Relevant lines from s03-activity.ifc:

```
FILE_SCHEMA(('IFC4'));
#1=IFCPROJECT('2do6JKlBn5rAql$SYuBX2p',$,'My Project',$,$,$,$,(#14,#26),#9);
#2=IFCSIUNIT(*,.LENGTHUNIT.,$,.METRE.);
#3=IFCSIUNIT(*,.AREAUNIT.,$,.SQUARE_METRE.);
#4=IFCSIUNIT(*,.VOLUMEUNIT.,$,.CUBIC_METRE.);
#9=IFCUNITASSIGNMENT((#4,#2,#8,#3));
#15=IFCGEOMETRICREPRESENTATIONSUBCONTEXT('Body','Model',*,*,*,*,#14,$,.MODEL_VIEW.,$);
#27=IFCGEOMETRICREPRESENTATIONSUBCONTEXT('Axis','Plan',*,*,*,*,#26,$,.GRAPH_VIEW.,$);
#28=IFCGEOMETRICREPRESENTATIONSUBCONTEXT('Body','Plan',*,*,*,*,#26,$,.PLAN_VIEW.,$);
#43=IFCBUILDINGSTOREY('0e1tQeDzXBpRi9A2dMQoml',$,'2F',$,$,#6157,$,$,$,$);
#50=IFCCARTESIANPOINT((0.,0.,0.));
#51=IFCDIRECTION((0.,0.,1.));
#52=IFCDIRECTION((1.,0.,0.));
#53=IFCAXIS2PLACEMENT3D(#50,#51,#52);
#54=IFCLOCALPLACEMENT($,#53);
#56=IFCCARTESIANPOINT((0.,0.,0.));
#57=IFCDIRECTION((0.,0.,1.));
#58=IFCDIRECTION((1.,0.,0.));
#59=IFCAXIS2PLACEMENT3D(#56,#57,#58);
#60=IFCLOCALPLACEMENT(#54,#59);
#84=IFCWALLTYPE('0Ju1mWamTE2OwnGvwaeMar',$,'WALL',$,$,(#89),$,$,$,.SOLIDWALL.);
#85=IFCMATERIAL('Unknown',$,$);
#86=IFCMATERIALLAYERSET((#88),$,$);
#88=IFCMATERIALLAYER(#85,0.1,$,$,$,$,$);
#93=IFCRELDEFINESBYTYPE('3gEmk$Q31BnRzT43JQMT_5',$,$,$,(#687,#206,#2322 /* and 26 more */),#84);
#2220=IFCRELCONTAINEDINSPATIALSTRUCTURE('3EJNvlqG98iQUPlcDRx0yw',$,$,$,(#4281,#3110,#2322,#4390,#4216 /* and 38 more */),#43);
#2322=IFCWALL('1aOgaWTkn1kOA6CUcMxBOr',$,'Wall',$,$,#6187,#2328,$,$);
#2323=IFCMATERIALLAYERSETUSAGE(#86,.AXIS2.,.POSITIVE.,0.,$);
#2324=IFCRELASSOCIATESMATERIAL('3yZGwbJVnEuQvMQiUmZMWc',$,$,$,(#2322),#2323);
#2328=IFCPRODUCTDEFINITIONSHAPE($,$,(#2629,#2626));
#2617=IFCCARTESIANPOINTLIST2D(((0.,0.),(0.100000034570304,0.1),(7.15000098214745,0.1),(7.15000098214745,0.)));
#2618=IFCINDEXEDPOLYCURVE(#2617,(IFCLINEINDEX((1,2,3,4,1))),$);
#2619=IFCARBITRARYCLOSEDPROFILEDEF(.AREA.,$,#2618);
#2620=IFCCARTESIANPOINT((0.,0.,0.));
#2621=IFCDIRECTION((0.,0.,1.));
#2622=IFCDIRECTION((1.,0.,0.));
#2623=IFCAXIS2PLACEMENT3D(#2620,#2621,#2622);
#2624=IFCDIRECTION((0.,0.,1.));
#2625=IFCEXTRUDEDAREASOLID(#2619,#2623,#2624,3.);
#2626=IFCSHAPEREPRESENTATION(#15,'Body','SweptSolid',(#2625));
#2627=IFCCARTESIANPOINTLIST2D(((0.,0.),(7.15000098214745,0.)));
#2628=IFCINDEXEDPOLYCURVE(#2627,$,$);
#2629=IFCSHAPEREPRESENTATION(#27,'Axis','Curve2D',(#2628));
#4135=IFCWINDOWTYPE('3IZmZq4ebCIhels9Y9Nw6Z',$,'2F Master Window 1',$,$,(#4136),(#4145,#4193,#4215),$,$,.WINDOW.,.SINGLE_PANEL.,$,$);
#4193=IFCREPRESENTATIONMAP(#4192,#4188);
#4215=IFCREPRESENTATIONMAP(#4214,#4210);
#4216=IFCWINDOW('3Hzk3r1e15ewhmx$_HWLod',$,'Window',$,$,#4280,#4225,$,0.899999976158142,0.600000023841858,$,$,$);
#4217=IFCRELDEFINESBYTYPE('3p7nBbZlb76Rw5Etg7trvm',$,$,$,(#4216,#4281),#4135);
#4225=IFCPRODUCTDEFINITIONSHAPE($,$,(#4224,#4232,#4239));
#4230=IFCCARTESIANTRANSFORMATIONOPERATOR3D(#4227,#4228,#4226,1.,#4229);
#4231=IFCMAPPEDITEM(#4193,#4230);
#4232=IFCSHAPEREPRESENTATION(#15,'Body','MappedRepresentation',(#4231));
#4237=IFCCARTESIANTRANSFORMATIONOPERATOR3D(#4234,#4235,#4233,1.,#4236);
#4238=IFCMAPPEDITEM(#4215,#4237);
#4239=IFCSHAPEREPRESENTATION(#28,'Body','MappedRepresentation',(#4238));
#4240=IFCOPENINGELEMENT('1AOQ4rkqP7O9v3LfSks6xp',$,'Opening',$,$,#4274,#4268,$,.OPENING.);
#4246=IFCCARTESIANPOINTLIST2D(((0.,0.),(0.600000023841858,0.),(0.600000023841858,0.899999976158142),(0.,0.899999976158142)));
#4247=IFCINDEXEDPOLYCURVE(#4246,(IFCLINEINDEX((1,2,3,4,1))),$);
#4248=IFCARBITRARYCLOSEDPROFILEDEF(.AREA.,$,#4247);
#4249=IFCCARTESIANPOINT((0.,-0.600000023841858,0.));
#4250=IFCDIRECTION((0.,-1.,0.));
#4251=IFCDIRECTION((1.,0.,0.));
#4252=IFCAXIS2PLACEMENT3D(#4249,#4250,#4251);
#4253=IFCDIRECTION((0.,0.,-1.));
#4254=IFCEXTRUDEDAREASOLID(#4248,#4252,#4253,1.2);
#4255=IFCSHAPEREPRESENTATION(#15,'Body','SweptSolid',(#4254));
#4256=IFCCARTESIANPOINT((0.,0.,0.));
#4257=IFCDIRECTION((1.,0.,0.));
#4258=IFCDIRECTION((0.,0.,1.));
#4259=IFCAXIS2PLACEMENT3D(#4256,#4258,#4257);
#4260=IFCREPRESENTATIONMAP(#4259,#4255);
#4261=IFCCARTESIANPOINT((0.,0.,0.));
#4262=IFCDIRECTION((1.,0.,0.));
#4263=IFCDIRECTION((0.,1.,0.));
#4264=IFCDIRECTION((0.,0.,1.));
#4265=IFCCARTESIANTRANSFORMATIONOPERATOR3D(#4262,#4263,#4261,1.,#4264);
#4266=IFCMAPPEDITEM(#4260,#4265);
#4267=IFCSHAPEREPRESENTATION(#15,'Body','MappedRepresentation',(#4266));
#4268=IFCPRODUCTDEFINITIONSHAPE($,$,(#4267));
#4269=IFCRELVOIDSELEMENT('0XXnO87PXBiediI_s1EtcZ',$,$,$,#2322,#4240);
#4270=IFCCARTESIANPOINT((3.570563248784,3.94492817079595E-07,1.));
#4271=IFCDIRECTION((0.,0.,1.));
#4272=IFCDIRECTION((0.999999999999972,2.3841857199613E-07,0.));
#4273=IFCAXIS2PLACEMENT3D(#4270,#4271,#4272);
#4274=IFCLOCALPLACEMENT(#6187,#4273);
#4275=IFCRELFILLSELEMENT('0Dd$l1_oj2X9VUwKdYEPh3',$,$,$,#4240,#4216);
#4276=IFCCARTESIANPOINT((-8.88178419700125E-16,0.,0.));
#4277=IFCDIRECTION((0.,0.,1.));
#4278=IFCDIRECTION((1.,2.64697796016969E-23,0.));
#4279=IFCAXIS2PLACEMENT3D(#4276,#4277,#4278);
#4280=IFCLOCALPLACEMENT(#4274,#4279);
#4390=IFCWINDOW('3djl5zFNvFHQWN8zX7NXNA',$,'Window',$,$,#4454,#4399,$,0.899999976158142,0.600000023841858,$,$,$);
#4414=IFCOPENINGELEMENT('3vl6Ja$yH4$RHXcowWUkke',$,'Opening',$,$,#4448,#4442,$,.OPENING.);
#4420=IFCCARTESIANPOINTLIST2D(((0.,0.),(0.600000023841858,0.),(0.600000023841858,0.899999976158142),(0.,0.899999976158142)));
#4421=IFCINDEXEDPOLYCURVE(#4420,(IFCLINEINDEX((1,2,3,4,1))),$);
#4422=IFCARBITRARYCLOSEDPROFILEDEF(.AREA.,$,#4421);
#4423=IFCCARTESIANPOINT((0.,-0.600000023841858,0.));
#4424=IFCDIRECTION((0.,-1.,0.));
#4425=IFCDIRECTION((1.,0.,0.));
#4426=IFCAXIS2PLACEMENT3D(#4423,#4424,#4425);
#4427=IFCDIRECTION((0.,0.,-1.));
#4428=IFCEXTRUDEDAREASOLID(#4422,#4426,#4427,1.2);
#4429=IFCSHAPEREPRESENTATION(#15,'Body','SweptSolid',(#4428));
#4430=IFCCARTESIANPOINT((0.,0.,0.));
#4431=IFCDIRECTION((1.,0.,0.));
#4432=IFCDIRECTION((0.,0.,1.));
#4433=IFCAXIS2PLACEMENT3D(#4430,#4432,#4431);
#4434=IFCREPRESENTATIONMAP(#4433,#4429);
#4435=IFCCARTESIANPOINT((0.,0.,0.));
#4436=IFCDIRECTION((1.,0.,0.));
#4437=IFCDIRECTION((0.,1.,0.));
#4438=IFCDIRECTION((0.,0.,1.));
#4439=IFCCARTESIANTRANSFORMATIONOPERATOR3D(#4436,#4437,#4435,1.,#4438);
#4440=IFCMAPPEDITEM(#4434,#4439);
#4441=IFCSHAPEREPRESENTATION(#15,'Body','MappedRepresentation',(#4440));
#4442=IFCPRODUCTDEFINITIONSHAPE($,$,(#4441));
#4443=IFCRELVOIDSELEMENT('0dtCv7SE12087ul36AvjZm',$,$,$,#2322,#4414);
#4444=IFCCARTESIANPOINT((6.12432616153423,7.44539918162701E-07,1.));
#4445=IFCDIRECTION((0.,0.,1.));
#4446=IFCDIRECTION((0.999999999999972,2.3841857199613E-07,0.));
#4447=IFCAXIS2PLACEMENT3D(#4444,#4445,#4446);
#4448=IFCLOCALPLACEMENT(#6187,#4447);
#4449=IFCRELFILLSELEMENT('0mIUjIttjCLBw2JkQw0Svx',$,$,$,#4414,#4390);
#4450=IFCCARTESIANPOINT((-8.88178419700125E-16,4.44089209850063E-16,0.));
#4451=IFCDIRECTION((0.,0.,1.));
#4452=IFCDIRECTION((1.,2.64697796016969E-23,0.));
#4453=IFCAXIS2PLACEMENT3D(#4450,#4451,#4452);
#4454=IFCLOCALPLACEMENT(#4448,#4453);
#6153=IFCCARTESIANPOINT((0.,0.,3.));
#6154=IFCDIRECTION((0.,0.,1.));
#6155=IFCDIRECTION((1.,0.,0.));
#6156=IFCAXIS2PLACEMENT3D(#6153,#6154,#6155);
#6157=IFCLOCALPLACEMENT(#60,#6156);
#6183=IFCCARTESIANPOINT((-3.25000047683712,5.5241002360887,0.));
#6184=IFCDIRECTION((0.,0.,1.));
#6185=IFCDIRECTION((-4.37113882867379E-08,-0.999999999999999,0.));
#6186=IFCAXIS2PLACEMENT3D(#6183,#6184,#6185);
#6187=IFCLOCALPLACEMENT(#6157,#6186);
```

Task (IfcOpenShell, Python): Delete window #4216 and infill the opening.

```python
import ifcopenshell
import ifcopenshell.api.feature
import ifcopenshell.api.root
import ifcopenshell.geom
import ifcopenshell.util.shape

model = ifcopenshell.open("s03-activity.ifc")
settings = ifcopenshell.geom.settings()


def volume(element):
    """Net volume in cubic metres, openings subtracted."""
    shape = ifcopenshell.geom.create_shape(settings, element)
    return ifcopenshell.util.shape.get_volume(shape.geometry)


window = model.by_guid("3Hzk3r1e15ewhmx$_HWLod")
opening = window.FillsVoids[0].RelatingOpeningElement
wall = opening.VoidsElements[0].RelatingBuildingElement
before = volume(wall)

ifcopenshell.api.root.remove_product(model, product=window)
ifcopenshell.api.feature.remove_feature(model, feature=opening)

after = volume(wall)

print(f"wall volume {before:.3f} -> {after:.3f} m3")

model.write("s03-activity-out.ifc")
```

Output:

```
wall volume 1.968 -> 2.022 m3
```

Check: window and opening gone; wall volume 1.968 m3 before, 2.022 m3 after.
